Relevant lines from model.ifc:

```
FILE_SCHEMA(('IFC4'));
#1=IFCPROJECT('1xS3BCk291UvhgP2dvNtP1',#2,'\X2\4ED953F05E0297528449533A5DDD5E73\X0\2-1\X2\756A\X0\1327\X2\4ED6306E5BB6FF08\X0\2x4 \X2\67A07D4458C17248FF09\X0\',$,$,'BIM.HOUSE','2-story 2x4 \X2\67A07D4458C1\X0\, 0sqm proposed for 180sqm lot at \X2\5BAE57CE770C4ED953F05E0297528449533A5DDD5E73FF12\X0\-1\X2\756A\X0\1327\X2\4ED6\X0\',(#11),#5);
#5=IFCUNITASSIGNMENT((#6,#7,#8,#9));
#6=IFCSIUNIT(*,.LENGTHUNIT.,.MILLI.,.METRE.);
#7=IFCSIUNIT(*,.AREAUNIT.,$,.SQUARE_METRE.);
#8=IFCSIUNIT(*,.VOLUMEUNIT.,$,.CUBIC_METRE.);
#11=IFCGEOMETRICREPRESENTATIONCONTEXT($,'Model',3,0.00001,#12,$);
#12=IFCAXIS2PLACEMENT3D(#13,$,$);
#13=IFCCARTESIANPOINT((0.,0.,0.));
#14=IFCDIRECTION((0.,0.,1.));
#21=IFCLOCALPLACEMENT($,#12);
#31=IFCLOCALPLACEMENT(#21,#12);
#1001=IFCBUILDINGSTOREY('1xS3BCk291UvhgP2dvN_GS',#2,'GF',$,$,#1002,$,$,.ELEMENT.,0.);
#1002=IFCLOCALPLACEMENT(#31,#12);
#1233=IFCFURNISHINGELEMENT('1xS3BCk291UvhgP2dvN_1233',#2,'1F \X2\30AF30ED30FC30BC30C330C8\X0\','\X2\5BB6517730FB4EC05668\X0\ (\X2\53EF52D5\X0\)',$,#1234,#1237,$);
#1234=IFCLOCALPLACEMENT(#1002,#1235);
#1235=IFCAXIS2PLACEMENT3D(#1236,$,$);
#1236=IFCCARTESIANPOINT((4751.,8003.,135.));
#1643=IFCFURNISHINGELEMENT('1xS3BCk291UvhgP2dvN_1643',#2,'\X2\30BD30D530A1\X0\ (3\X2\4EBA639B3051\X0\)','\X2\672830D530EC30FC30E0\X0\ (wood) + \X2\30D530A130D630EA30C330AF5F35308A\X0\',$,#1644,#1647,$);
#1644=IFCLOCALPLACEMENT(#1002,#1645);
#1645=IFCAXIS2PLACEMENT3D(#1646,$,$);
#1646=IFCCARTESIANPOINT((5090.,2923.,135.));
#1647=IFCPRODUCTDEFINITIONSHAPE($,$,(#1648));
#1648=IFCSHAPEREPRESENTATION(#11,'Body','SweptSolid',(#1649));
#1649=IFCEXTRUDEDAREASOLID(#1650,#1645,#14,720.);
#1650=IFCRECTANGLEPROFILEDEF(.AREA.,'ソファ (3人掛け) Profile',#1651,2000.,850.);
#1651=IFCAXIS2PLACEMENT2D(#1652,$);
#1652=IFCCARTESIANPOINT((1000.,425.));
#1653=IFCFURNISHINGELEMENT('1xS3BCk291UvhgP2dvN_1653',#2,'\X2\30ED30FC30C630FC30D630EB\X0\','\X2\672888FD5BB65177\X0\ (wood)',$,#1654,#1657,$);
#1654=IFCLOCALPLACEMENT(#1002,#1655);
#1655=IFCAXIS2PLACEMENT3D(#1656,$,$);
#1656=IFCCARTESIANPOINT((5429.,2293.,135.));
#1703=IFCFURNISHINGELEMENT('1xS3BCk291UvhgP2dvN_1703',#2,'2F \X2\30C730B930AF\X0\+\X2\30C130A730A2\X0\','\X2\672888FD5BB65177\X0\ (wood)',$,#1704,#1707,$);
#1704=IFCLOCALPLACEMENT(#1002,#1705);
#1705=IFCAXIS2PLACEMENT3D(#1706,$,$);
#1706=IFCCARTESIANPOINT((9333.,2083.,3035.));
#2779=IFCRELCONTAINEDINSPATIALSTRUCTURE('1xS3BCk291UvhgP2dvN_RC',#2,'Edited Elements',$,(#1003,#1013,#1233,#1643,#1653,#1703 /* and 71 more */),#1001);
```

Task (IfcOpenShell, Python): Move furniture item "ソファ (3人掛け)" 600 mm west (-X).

```python
import ifcopenshell
import ifcopenshell.api.geometry
import ifcopenshell.util.placement

model = ifcopenshell.open("model.ifc")

item = model.by_id(1643)
matrix = ifcopenshell.util.placement.get_local_placement(item.ObjectPlacement)
matrix[0, 3] -= 600.0
ifcopenshell.api.geometry.edit_object_placement(model, product=item, matrix=matrix, is_si=False)

print(ifcopenshell.util.placement.get_local_placement(item.ObjectPlacement).round(3) + 0.0)

model.write("model-out.ifc")
```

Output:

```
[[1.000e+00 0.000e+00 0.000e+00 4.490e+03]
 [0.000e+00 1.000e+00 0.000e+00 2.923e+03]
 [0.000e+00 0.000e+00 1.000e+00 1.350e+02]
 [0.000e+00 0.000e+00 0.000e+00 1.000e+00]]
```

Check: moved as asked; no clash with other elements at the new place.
